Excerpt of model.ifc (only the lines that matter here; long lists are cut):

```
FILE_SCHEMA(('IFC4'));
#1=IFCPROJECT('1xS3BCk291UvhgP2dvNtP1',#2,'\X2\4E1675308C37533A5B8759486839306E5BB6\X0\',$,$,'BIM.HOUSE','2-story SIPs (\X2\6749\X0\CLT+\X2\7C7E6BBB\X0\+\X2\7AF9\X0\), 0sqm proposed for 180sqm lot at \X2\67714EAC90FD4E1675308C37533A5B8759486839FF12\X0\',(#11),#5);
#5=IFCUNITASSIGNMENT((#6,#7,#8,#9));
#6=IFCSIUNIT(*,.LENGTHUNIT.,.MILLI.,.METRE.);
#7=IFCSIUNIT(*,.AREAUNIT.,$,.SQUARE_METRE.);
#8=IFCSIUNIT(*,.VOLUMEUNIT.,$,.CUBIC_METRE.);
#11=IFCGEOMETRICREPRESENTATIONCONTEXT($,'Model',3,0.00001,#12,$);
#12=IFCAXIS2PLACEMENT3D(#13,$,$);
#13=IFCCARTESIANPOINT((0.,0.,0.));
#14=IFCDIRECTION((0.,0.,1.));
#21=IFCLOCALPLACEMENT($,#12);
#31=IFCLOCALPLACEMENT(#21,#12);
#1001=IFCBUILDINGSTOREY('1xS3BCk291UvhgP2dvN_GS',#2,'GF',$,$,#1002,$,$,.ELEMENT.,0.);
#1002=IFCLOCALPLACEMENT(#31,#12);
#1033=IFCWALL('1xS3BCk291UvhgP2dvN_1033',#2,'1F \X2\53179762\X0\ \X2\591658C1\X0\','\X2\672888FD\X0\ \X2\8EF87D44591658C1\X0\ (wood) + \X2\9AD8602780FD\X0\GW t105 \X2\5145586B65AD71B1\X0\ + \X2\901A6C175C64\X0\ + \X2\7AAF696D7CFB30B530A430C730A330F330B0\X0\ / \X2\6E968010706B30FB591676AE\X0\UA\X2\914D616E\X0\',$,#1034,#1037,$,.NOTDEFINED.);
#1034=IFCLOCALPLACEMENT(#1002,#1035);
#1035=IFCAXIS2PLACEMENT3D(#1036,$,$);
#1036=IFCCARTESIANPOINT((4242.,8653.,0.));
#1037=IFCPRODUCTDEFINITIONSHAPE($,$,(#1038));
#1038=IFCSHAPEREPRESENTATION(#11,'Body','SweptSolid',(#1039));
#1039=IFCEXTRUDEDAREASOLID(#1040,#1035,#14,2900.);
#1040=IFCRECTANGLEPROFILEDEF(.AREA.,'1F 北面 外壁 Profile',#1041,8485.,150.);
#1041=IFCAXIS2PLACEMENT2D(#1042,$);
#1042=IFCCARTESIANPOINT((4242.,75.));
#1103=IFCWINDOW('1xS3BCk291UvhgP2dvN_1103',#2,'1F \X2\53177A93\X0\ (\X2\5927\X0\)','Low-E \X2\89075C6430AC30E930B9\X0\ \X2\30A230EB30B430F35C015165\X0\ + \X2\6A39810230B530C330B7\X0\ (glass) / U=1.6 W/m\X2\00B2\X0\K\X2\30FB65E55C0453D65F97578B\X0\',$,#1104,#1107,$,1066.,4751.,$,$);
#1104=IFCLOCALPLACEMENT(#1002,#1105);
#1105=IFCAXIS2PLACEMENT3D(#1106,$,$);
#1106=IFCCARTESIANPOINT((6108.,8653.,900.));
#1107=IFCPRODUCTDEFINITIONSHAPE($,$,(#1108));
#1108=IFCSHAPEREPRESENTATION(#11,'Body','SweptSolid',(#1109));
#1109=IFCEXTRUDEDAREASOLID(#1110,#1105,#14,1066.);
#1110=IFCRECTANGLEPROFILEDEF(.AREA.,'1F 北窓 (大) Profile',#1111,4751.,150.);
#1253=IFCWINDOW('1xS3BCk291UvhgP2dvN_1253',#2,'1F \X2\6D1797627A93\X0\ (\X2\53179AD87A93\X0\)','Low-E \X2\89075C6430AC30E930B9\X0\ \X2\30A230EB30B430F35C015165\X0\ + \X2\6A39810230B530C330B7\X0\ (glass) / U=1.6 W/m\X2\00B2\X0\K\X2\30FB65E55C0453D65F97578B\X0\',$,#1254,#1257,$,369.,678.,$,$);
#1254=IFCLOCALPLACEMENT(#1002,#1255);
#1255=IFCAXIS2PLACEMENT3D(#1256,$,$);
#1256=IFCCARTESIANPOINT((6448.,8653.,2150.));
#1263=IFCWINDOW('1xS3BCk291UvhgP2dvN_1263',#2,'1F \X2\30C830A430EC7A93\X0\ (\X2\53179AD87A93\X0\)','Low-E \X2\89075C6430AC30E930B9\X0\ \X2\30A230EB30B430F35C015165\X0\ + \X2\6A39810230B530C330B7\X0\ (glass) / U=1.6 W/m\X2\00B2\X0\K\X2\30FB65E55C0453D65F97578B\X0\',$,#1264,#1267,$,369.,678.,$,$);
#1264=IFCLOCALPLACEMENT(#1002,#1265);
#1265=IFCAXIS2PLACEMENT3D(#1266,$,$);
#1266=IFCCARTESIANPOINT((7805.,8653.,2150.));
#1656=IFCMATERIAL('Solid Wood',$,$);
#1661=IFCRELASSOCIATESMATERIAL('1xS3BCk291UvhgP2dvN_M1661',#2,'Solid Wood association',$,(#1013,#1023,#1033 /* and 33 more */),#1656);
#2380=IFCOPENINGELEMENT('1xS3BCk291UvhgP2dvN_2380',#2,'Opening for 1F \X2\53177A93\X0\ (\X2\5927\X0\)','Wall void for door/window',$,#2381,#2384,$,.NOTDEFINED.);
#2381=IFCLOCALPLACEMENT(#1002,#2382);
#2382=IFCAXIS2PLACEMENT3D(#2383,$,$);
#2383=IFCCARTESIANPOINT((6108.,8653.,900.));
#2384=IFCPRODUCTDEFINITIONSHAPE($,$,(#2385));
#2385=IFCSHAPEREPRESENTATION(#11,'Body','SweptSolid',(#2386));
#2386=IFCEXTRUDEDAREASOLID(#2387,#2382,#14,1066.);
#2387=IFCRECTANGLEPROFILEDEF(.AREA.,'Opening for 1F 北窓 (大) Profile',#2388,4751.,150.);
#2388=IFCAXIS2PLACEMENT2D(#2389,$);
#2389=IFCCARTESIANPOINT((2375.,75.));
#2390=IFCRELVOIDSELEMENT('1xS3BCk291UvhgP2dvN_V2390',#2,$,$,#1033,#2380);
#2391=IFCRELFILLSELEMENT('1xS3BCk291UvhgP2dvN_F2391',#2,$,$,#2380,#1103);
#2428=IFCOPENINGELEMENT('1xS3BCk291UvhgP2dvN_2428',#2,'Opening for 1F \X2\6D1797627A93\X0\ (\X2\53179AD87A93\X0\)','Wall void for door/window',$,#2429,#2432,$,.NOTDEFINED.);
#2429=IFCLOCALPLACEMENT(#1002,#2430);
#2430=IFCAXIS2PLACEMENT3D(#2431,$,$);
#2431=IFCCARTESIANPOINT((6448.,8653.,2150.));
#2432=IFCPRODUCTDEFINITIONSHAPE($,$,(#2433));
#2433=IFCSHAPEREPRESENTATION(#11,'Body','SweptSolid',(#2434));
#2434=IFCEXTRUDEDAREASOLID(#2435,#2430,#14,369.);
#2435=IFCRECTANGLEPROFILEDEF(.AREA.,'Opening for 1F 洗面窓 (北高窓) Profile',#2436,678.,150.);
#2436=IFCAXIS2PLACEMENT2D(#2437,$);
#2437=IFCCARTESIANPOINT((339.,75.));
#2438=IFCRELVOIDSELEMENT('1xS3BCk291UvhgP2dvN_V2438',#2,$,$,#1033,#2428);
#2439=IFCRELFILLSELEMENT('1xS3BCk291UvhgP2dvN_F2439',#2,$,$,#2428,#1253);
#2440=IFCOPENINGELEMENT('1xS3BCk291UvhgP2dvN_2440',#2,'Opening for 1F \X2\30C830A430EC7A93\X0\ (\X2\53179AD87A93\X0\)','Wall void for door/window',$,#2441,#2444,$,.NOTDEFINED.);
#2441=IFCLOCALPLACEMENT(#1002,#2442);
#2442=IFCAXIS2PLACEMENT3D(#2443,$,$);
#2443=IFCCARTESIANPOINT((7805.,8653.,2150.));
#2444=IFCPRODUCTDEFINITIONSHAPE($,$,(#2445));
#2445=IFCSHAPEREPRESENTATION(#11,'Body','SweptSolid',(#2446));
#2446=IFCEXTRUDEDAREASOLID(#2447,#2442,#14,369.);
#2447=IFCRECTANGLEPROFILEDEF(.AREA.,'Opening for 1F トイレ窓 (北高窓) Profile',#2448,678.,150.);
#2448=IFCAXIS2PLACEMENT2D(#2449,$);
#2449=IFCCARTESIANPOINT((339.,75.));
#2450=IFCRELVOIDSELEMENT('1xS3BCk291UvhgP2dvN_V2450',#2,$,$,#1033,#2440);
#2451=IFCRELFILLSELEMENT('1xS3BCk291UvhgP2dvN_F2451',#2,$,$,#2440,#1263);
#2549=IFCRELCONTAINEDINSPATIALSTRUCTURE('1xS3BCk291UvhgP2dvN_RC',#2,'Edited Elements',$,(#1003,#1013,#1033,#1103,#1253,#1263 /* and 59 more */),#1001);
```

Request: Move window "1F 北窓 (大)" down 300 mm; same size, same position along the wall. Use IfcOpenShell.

```python
import numpy as np
import ifcopenshell
import ifcopenshell.api.geometry
import ifcopenshell.util.placement
import ifcopenshell.util.unit

model = ifcopenshell.open("model.ifc")
unit_scale = ifcopenshell.util.unit.calculate_unit_scale(model)

window = model.by_guid("1xS3BCk291UvhgP2dvN_1103")
opening = window.FillsVoids[0].RelatingOpeningElement
dz = -300.0

shift = np.array([0.0, 0.0, dz])
# The window is not placed relative to its opening, so move both.
for product in (opening, window):
    matrix = ifcopenshell.util.placement.get_local_placement(product.ObjectPlacement)
    matrix[:3, 3] += shift
    ifcopenshell.api.geometry.edit_object_placement(model, product=product, matrix=matrix, is_si=False)

print(f"moved by {dz * unit_scale:+.3f} m")

model.write("model-out.ifc")
```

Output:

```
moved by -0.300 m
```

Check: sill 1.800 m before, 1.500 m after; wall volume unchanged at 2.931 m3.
